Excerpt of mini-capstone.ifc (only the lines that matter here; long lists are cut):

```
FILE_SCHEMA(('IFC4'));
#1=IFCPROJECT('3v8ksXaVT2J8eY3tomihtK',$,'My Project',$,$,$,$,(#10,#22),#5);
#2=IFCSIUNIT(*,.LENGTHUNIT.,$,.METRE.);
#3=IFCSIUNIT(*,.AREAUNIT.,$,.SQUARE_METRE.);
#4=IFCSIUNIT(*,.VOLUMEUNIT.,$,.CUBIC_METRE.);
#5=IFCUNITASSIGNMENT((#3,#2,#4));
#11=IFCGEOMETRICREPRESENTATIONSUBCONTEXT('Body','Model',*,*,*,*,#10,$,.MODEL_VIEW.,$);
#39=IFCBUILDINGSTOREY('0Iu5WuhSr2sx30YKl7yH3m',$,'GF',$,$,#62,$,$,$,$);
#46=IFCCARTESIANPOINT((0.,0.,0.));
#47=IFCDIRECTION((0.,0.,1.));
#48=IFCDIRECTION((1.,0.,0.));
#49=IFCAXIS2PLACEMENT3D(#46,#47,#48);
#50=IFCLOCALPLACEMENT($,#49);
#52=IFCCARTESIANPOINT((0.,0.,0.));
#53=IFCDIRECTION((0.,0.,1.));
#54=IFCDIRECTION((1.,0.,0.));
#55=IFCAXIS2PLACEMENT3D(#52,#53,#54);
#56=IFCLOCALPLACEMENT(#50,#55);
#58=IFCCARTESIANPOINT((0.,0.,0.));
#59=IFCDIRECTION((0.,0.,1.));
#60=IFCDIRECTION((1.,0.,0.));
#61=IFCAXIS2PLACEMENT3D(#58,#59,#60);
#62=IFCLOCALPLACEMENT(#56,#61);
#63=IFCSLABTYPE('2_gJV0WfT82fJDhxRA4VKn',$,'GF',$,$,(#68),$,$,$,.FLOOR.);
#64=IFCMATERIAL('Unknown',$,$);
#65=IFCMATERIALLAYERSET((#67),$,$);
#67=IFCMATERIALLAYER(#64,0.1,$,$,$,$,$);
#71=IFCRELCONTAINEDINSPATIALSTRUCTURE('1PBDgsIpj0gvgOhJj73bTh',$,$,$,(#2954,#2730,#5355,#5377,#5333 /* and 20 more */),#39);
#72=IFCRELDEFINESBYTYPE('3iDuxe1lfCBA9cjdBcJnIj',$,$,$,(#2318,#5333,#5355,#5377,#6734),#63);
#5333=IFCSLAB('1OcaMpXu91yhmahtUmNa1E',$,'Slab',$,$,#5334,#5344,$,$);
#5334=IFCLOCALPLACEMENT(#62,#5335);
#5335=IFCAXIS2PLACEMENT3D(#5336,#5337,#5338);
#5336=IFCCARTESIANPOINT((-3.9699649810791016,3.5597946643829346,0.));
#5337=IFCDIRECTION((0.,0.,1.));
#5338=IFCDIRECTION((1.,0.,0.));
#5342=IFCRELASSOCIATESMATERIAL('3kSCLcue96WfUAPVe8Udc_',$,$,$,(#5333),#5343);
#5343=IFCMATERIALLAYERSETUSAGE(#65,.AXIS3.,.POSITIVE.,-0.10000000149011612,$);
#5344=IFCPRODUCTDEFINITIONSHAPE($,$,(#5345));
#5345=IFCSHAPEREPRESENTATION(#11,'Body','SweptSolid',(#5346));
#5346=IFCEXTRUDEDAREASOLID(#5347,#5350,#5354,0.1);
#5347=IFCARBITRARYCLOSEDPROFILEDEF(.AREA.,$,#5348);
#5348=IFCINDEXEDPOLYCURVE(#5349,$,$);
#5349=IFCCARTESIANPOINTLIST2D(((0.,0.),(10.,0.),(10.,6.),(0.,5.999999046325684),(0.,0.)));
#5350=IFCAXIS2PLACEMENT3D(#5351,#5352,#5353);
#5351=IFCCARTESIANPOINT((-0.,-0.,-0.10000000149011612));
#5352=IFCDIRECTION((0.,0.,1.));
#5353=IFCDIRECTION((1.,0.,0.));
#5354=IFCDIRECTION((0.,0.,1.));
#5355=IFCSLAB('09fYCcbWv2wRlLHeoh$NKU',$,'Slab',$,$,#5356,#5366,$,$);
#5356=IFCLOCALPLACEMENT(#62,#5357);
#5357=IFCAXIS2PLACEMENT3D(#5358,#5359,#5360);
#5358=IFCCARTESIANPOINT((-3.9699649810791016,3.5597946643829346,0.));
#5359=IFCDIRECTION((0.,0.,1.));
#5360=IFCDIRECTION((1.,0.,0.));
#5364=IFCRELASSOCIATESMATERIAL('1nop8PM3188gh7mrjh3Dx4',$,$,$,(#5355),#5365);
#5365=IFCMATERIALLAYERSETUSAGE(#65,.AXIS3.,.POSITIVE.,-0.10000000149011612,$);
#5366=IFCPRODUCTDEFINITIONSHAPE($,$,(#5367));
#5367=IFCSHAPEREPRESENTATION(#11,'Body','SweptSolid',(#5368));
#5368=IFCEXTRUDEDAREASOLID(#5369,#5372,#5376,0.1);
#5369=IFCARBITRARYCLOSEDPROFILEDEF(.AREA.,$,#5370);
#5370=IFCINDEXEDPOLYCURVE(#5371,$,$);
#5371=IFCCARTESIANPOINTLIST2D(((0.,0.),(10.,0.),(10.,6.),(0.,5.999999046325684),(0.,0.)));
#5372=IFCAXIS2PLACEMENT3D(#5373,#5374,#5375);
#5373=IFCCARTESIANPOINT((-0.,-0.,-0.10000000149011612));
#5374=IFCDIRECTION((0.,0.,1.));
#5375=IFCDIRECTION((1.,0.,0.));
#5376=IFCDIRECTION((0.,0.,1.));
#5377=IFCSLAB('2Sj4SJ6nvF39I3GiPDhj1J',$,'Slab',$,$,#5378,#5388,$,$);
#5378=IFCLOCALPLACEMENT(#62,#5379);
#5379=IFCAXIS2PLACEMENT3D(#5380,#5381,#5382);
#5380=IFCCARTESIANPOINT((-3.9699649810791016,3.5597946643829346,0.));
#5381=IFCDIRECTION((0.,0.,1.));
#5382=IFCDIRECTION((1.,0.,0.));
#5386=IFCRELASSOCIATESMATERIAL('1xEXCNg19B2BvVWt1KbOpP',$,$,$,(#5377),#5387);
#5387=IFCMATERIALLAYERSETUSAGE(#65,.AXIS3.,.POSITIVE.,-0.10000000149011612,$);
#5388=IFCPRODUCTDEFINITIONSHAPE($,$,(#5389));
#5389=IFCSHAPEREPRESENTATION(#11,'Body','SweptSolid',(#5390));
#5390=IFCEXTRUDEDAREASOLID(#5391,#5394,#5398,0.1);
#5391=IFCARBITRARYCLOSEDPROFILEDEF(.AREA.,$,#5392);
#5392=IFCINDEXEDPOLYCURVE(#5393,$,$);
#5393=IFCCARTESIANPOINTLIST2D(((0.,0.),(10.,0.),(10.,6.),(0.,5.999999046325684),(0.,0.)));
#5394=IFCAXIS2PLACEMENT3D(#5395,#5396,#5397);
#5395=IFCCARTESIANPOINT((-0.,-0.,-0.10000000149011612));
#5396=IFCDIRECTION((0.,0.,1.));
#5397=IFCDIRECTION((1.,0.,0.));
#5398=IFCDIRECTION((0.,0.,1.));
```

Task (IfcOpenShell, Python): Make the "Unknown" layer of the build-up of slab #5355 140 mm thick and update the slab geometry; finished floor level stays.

```python
import ifcopenshell
import ifcopenshell.util.element
import ifcopenshell.util.representation
import ifcopenshell.util.unit

model = ifcopenshell.open("mini-capstone.ifc")
unit_scale = ifcopenshell.util.unit.calculate_unit_scale(model)

layer_set = model.by_id(65)
layer = next(l for l in layer_set.MaterialLayers if l.Material and l.Material.Name == "Unknown")
change = 0.14 / unit_scale - layer.LayerThickness
layer.LayerThickness += change

# The layer set is shared, so every slab that uses it gets the new thickness.
slabs = [e for e in ifcopenshell.util.element.get_elements_by_material(model, layer_set) if e.is_a("IfcSlab")]
for slab in sorted(slabs, key=lambda e: e.id()):
    body = ifcopenshell.util.representation.get_representation(slab, "Model", "Body")
    solid = body.Items[0]
    old_depth = solid.Depth
    solid.Depth += change
    # Extruded upwards: lower the start of the extrusion so the top stays.
    x, y, z = solid.Position.Location.Coordinates
    solid.Position.Location = model.createIfcCartesianPoint((x, y, z - change))
    print(slab.id(), f"{old_depth:g} -> {solid.Depth:g}")

# The layers are counted up from the underside, which has moved.
for usage in {ifcopenshell.util.element.get_material(slab) for slab in slabs}:
    usage.OffsetFromReferenceLine -= change

model.write("mini-capstone-out.ifc")
```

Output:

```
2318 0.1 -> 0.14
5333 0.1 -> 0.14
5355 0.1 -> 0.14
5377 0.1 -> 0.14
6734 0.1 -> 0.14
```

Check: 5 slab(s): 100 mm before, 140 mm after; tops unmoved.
